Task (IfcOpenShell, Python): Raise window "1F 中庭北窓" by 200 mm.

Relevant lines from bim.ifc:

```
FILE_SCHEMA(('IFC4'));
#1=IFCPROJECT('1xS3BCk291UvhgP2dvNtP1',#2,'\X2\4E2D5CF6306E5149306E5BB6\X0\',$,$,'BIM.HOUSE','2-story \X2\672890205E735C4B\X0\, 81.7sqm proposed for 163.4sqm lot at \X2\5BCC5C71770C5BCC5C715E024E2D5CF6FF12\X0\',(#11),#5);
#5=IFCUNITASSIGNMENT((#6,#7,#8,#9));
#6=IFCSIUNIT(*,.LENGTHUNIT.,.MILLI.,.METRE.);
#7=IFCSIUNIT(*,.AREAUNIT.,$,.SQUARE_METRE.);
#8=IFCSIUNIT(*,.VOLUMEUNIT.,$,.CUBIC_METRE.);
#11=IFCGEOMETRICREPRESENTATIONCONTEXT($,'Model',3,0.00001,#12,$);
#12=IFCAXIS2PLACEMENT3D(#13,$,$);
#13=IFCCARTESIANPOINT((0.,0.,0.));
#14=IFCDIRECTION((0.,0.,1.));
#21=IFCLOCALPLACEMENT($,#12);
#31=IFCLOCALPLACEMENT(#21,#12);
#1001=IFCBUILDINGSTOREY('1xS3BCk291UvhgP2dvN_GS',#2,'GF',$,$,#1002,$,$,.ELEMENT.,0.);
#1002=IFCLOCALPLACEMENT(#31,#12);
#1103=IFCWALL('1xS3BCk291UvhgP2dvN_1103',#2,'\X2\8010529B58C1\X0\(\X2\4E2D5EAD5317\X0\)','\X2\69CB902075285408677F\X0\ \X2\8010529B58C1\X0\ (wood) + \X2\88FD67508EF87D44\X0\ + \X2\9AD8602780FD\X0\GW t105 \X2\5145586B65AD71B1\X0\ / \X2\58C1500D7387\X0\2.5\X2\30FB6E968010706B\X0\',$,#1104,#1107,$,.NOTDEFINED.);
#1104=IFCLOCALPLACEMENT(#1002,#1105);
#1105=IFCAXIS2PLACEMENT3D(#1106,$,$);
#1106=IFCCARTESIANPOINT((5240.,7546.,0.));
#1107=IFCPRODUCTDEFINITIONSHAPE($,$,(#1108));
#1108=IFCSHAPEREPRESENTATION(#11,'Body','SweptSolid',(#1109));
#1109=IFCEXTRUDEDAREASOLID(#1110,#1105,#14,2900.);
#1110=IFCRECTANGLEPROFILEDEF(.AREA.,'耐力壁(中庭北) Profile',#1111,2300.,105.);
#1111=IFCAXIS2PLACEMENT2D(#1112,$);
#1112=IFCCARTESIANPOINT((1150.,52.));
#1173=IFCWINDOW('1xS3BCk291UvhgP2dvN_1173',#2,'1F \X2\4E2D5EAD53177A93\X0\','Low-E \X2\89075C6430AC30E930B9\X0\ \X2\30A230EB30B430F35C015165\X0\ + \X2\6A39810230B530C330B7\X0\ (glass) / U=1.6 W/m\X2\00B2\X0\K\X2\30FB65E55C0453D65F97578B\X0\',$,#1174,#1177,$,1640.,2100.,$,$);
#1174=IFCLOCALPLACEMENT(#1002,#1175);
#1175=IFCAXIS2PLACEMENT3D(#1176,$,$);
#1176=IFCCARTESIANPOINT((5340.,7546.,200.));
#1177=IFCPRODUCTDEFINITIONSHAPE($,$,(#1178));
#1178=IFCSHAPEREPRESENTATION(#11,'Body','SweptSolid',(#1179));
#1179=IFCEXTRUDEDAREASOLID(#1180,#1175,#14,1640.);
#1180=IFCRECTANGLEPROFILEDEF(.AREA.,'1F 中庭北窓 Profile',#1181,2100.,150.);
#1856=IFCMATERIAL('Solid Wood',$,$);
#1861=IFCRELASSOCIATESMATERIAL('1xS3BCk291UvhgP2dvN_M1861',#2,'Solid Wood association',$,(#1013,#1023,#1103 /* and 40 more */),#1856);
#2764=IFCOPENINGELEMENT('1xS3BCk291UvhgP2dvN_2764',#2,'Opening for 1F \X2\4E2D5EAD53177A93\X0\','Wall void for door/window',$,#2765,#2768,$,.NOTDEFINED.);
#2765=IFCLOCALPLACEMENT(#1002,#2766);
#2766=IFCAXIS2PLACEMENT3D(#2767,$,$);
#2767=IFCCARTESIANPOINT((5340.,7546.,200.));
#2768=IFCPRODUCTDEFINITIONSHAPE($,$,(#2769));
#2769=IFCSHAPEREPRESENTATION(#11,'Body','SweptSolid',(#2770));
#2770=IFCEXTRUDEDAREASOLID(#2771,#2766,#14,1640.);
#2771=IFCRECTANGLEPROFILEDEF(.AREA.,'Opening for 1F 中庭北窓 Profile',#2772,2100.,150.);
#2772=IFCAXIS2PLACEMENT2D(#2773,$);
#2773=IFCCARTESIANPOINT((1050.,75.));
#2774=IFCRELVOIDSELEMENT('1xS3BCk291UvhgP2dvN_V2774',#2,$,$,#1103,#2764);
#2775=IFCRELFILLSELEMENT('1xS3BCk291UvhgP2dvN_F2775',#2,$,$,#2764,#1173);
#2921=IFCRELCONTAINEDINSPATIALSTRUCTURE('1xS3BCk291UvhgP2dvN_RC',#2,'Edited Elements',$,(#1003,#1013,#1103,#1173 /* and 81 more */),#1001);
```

```python
import numpy as np
import ifcopenshell
import ifcopenshell.api.geometry
import ifcopenshell.util.placement
import ifcopenshell.util.unit

model = ifcopenshell.open("bim.ifc")
unit_scale = ifcopenshell.util.unit.calculate_unit_scale(model)

window = model.by_guid("1xS3BCk291UvhgP2dvN_1173")
opening = window.FillsVoids[0].RelatingOpeningElement
dz = 0.2 / unit_scale

shift = np.array([0.0, 0.0, dz])
# The window is not placed relative to its opening, so move both.
for product in (opening, window):
    matrix = ifcopenshell.util.placement.get_local_placement(product.ObjectPlacement)
    matrix[:3, 3] += shift
    ifcopenshell.api.geometry.edit_object_placement(model, product=product, matrix=matrix, is_si=False)

print(f"moved by {dz * unit_scale:+.3f} m")

model.write("bim_edited.ifc")
```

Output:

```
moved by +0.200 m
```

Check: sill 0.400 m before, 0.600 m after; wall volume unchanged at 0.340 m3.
